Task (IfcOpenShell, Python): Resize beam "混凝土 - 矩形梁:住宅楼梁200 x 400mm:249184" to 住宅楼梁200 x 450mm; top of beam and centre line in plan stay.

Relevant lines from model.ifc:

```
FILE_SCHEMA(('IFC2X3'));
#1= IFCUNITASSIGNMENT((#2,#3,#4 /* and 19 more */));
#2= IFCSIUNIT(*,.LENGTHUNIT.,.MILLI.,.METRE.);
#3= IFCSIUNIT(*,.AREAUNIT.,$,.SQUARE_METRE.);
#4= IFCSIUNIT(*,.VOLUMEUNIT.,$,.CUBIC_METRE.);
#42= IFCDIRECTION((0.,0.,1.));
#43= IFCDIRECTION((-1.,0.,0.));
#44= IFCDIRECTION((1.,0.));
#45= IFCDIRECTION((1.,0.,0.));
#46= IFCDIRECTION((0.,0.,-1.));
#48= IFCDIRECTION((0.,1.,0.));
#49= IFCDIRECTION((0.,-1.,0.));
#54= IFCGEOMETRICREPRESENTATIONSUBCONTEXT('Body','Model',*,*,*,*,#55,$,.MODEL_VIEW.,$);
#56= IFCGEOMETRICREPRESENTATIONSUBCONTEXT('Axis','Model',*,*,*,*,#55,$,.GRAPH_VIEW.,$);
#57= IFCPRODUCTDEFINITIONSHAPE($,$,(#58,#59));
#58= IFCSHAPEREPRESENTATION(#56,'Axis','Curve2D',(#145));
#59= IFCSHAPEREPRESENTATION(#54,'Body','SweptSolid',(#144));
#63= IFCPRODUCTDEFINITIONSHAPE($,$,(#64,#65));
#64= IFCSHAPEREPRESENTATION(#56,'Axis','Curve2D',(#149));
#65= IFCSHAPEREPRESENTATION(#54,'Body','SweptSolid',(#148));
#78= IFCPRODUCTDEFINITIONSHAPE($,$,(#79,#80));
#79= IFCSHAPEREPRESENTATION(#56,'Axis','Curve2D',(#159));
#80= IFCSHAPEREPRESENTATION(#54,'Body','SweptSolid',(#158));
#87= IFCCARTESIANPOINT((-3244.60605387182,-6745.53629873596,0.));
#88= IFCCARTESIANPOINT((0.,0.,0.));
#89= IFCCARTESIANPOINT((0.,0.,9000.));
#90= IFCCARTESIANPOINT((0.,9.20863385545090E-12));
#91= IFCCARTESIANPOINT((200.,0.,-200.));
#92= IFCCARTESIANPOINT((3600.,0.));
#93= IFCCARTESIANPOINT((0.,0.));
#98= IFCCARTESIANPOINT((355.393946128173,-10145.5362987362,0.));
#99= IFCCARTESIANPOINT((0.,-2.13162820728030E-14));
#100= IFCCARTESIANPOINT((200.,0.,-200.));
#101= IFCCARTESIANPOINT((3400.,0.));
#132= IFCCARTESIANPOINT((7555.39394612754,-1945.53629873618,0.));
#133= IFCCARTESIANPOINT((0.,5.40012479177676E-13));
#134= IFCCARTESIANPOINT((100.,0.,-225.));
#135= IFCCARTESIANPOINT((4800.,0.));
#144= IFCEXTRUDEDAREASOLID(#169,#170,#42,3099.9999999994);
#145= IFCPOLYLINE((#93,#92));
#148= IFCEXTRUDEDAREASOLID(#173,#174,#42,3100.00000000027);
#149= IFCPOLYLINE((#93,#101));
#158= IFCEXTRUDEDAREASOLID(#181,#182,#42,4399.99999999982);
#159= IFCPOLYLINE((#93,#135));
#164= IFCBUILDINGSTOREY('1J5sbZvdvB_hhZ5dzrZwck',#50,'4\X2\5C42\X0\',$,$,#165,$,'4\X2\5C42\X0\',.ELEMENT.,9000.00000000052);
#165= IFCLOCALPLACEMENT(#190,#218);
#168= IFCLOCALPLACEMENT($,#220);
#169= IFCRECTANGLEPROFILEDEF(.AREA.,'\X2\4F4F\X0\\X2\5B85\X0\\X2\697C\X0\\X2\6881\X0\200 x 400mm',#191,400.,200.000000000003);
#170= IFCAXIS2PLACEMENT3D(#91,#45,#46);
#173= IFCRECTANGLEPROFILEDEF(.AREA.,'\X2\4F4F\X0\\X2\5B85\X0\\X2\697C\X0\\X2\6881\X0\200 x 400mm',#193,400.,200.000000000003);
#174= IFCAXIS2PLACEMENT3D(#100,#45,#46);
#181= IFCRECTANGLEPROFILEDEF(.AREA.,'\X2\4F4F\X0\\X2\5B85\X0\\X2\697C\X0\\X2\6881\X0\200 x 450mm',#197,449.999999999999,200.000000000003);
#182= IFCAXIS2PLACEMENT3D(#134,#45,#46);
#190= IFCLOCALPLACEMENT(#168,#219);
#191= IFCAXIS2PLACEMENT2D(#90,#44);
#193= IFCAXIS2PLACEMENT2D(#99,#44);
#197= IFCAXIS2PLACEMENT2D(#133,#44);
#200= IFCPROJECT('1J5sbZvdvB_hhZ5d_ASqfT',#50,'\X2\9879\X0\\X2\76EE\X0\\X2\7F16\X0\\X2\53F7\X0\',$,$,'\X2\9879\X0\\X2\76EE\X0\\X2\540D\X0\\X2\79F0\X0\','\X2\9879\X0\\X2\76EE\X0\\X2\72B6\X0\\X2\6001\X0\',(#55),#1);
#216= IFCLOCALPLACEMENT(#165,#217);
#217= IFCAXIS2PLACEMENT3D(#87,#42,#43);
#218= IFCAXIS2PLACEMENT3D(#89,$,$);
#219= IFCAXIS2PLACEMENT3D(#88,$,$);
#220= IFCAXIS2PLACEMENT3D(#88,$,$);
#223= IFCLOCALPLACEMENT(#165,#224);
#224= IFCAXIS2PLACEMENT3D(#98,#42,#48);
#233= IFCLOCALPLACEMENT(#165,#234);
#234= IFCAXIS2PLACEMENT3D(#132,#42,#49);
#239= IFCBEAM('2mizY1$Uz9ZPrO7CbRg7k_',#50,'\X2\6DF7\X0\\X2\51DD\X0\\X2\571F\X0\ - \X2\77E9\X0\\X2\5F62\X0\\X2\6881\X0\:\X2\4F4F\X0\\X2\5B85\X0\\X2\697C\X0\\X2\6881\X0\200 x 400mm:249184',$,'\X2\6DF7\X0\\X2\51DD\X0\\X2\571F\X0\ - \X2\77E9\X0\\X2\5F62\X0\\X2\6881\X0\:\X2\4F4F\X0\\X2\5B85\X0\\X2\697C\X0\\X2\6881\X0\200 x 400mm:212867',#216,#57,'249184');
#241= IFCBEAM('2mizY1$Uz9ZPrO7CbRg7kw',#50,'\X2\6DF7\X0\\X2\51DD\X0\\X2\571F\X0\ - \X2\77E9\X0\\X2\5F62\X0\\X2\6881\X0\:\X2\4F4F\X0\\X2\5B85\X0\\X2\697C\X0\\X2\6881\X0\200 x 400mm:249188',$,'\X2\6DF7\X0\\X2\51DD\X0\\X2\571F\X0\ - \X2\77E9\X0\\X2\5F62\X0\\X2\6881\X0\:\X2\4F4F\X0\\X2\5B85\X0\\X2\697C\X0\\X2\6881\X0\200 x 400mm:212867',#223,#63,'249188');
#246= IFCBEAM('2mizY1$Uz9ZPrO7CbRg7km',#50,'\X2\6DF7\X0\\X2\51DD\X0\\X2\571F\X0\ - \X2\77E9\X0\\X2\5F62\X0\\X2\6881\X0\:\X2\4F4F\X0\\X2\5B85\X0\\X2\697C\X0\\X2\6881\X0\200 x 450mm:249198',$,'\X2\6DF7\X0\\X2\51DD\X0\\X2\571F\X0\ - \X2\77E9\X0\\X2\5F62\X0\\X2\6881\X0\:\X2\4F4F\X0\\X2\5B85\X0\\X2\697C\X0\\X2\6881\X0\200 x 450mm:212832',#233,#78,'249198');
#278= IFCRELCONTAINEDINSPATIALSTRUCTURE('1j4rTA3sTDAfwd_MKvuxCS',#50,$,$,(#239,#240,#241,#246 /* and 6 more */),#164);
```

```python
import ifcopenshell
import ifcopenshell.util.element
import ifcopenshell.util.representation

model = ifcopenshell.open("model.ifc")

member = model.by_guid("2mizY1$Uz9ZPrO7CbRg7k_")
source = next(p for p in model.by_type("IfcRectangleProfileDef") if p.ProfileName == "住宅楼梁200 x 450mm")

body = ifcopenshell.util.representation.get_representation(member, "Model", "Body")
solid = body.Items[0]
old_profile = solid.SweptArea

# Copy the section's sizes but keep this member's own profile position.
profile = ifcopenshell.util.element.copy(model, source)
# Profiles are centred, so shift by half the change in depth to hold the top.
shift = (old_profile.XDim - profile.XDim) / 2
x, y = old_profile.Position.Location.Coordinates
up = (-1.0, 0.0)  # upwards, in the solid's own plane
location = model.createIfcCartesianPoint((x + up[0] * shift, y + up[1] * shift))
profile.Position = model.createIfcAxis2Placement2D(location, old_profile.Position.RefDirection)
solid.SweptArea = profile
if not model.get_total_inverses(old_profile):
    ifcopenshell.util.element.remove_deep2(model, old_profile)
member.Name = member.Name.replace("住宅楼梁200 x 400mm", "住宅楼梁200 x 450mm")
member.ObjectType = member.ObjectType.replace("住宅楼梁200 x 400mm", "住宅楼梁200 x 450mm")

print(solid.SweptArea)

model.write("model_updated.ifc")
```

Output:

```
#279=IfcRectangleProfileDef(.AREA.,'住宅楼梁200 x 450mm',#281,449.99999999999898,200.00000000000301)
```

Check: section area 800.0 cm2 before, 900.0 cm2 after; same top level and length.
